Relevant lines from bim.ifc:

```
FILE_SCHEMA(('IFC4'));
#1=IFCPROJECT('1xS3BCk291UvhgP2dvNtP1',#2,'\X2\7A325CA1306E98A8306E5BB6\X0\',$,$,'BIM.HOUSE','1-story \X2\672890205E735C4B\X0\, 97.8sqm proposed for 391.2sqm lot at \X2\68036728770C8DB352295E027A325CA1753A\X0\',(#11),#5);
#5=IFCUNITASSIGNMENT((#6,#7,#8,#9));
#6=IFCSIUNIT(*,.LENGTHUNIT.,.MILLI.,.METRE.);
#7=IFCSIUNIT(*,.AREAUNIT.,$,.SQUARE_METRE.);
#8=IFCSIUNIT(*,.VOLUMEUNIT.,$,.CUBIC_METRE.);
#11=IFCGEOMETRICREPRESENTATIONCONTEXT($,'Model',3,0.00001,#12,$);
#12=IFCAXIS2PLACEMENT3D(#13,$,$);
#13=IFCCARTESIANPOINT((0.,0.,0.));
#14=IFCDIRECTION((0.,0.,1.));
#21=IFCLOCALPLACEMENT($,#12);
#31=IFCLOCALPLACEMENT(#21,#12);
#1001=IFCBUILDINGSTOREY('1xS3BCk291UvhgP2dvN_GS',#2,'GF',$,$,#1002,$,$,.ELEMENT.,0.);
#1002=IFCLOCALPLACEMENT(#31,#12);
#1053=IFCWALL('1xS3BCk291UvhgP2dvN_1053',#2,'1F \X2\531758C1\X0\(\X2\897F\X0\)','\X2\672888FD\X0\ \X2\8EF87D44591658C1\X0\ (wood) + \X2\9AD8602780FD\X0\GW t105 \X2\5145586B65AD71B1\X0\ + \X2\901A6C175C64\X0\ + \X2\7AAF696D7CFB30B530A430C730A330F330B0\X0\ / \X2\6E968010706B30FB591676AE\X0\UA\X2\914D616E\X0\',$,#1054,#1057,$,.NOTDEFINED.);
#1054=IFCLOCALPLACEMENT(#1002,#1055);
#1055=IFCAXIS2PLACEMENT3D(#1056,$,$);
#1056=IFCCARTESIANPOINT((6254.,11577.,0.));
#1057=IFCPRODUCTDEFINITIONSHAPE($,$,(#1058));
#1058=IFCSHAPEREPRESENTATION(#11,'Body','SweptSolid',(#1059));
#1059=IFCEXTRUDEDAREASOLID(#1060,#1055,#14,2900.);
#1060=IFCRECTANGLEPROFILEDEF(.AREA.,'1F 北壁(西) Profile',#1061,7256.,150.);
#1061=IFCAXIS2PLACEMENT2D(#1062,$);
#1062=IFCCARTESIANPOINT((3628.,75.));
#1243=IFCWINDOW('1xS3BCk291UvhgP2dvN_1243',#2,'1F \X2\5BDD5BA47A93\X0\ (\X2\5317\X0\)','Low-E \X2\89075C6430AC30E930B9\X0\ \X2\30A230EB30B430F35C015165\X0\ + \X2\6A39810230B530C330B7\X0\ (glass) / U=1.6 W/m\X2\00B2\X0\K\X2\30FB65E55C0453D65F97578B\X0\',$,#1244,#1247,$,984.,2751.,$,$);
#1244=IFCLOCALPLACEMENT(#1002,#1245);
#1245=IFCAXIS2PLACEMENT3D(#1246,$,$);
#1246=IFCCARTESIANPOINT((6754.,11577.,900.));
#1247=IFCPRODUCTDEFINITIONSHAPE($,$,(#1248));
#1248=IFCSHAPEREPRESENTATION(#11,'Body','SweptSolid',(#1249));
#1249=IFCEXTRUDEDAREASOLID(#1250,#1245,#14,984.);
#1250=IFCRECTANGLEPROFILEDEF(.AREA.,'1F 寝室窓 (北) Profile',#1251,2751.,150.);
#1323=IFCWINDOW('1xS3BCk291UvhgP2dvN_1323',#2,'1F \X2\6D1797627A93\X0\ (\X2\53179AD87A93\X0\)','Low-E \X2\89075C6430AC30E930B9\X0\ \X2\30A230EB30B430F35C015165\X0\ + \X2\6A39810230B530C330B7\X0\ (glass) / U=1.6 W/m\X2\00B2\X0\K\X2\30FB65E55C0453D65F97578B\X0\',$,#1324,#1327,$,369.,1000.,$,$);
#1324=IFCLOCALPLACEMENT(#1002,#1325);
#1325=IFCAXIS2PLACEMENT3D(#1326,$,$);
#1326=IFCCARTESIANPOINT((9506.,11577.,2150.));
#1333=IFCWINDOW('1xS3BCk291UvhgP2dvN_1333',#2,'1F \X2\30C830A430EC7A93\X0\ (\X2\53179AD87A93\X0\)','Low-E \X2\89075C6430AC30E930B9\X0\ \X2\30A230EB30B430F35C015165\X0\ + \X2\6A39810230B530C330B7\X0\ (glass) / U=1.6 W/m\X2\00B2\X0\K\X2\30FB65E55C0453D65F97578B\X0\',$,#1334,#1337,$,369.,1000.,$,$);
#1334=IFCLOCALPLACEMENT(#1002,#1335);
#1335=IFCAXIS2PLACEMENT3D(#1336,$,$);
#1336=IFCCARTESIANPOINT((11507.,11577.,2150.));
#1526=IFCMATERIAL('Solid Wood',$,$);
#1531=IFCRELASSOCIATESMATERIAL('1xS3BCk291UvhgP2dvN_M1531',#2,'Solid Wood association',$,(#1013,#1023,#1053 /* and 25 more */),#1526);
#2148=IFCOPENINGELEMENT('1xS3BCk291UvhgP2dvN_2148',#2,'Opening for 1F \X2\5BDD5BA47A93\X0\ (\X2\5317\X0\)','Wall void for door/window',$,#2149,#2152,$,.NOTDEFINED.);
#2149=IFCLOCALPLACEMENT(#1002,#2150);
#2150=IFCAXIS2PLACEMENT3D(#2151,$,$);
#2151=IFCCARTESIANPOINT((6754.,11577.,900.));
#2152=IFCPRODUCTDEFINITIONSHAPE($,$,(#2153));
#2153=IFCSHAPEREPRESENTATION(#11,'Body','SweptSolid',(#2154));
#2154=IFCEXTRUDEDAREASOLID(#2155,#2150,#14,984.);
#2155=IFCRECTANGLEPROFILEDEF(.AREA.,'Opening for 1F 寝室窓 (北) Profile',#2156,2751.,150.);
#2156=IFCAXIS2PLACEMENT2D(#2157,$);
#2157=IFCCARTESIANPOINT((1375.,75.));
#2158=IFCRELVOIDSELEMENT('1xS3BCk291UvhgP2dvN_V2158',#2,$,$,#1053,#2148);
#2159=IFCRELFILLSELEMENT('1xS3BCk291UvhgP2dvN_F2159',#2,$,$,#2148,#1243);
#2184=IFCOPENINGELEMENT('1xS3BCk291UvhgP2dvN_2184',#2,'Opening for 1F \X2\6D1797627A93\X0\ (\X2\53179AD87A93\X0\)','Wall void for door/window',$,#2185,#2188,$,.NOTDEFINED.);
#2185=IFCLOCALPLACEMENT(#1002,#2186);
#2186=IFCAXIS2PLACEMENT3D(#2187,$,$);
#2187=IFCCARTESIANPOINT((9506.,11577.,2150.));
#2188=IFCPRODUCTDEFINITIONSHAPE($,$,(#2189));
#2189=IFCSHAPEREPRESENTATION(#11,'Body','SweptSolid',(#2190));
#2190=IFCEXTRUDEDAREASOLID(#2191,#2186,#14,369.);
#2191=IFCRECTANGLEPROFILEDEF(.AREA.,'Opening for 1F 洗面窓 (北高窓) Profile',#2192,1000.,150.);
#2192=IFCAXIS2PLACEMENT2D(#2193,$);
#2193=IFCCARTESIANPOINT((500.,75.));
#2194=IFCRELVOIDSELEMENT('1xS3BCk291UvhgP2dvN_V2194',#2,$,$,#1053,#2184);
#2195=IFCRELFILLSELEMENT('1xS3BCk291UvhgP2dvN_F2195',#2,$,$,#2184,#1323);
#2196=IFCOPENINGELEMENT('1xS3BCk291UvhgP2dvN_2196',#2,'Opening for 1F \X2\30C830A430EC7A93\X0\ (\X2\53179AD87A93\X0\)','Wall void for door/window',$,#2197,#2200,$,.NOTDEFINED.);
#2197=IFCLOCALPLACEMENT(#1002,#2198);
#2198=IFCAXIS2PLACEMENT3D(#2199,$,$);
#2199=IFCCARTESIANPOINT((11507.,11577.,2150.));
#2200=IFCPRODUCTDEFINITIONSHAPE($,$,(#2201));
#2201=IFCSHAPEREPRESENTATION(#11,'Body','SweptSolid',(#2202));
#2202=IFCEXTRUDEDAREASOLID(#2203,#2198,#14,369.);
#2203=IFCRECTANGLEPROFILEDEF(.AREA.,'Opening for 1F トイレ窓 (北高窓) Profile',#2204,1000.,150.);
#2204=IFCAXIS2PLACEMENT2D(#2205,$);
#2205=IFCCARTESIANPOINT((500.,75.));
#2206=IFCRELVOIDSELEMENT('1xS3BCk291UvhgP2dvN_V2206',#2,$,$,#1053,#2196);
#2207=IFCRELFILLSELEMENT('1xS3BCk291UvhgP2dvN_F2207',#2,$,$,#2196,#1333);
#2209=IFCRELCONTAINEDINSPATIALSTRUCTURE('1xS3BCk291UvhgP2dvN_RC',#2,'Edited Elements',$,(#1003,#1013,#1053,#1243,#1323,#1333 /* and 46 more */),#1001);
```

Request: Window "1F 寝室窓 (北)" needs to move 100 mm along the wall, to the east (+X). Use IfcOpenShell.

```python
import ifcopenshell
import ifcopenshell.api.geometry
import ifcopenshell.util.placement

model = ifcopenshell.open("bim.ifc")

window = model.by_id(1243)
opening = window.FillsVoids[0].RelatingOpeningElement
wall = opening.VoidsElements[0].RelatingBuildingElement

wall_matrix = ifcopenshell.util.placement.get_local_placement(wall.ObjectPlacement)
shift = wall_matrix[:3, 0] * 100.0
before = ifcopenshell.util.placement.get_local_placement(window.ObjectPlacement)[:3, 3].copy()

# The window is not placed relative to its opening, so move both.
for product in (opening, window):
    matrix = ifcopenshell.util.placement.get_local_placement(product.ObjectPlacement)
    matrix[:3, 3] += shift
    ifcopenshell.api.geometry.edit_object_placement(model, product=product, matrix=matrix, is_si=False)

after = ifcopenshell.util.placement.get_local_placement(window.ObjectPlacement)[:3, 3]
print("window moved by", (after - before).round(3) + 0.0)

model.write("bim_v2.ifc")
```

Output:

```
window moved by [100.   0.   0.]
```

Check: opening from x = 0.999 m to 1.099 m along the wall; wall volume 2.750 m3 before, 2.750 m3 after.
